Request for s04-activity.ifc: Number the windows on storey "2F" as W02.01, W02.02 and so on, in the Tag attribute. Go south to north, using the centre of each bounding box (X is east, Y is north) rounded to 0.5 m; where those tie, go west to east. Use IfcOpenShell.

First a look at what the model holds.

```python
import ifcopenshell
import ifcopenshell.util.element
import ifcopenshell.util.placement

model = ifcopenshell.open("s04-activity.ifc")
print(model.schema)
storey = next(s for s in model.by_type("IfcBuildingStorey") if s.Name == "2F")
windows = [e for e in ifcopenshell.util.element.get_decomposition(storey) if e.is_a("IfcWindow")]
for e in sorted(windows, key=lambda e: e.id()):
    origin = ifcopenshell.util.placement.get_local_placement(e.ObjectPlacement)[:3, 3]
    print(e.id(), e.Tag, e.Name, origin.round(2) + 0.0, sep=" | ")
```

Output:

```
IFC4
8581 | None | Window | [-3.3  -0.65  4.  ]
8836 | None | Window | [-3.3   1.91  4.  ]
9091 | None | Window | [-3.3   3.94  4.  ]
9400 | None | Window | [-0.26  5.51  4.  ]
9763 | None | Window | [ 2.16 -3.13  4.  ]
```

```python
import ifcopenshell
import ifcopenshell.geom
import ifcopenshell.util.element
import ifcopenshell.util.shape

model = ifcopenshell.open("s04-activity.ifc")
settings = ifcopenshell.geom.settings()
settings.set("use-world-coords", True)


def centre(element):
    shape = ifcopenshell.geom.create_shape(settings, element)
    return ifcopenshell.util.shape.get_bbox_centroid(shape.geometry)


storey = next(s for s in model.by_type("IfcBuildingStorey") if s.Name == "2F")
windows = [e for e in ifcopenshell.util.element.get_decomposition(storey) if e.is_a("IfcWindow")]

# Insertion points can sit at a corner or the storey origin, so sort by the geometry (in metres).
centres = {e: centre(e) for e in windows}
windows.sort(key=lambda e: (round(centres[e][1] / 0.5), centres[e][0]))

for i, e in enumerate(windows, start=1):
    number = f"W02.{i:02d}"
    e.Tag = number
    print(e.id(), number)

model.write("s04-activity_edited.ifc")
```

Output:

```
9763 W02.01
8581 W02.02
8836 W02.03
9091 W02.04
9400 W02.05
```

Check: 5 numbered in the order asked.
